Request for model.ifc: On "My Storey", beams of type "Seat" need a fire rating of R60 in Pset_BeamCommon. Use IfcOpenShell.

First a look at what the model holds.

```python
import ifcopenshell
import ifcopenshell.util.element

model = ifcopenshell.open("model.ifc")
print(model.schema)
storey = next(s for s in model.by_type("IfcBuildingStorey") if s.Name == "My Storey")
beams = [e for e in ifcopenshell.util.element.get_decomposition(storey) if e.is_a("IfcBeam")]
seen = {}
for e in beams:
    element_type = ifcopenshell.util.element.get_type(e)
    key = (element_type.Name if element_type != e and element_type else None, ifcopenshell.util.element.get_pset(e, "Pset_BeamCommon", "FireRating"))
    seen[key] = seen.get(key, 0) + 1
for (name, value), count in sorted(seen.items(), key=str):
    print(count, "x", name, "|", value)
```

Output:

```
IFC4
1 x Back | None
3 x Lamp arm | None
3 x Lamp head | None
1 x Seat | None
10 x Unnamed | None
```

```python
import ifcopenshell
import ifcopenshell.api.pset
import ifcopenshell.util.element

model = ifcopenshell.open("model.ifc")

storey = next(s for s in model.by_type("IfcBuildingStorey") if s.Name == "My Storey")
beams = [e for e in ifcopenshell.util.element.get_decomposition(storey) if e.is_a("IfcBeam")]

count = 0
for e in beams:
    element_type = ifcopenshell.util.element.get_type(e)
    if element_type in (None, e) or element_type.Name != "Seat":
        continue
    # add_pset returns the element's existing set when there is one.
    pset = ifcopenshell.api.pset.add_pset(model, product=e, name="Pset_BeamCommon")
    ifcopenshell.api.pset.edit_pset(model, pset=pset, properties={"FireRating": "R60"})
    count += 1

print(count, "beams updated")

model.write("model_updated.ifc")
```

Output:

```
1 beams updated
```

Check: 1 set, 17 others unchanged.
